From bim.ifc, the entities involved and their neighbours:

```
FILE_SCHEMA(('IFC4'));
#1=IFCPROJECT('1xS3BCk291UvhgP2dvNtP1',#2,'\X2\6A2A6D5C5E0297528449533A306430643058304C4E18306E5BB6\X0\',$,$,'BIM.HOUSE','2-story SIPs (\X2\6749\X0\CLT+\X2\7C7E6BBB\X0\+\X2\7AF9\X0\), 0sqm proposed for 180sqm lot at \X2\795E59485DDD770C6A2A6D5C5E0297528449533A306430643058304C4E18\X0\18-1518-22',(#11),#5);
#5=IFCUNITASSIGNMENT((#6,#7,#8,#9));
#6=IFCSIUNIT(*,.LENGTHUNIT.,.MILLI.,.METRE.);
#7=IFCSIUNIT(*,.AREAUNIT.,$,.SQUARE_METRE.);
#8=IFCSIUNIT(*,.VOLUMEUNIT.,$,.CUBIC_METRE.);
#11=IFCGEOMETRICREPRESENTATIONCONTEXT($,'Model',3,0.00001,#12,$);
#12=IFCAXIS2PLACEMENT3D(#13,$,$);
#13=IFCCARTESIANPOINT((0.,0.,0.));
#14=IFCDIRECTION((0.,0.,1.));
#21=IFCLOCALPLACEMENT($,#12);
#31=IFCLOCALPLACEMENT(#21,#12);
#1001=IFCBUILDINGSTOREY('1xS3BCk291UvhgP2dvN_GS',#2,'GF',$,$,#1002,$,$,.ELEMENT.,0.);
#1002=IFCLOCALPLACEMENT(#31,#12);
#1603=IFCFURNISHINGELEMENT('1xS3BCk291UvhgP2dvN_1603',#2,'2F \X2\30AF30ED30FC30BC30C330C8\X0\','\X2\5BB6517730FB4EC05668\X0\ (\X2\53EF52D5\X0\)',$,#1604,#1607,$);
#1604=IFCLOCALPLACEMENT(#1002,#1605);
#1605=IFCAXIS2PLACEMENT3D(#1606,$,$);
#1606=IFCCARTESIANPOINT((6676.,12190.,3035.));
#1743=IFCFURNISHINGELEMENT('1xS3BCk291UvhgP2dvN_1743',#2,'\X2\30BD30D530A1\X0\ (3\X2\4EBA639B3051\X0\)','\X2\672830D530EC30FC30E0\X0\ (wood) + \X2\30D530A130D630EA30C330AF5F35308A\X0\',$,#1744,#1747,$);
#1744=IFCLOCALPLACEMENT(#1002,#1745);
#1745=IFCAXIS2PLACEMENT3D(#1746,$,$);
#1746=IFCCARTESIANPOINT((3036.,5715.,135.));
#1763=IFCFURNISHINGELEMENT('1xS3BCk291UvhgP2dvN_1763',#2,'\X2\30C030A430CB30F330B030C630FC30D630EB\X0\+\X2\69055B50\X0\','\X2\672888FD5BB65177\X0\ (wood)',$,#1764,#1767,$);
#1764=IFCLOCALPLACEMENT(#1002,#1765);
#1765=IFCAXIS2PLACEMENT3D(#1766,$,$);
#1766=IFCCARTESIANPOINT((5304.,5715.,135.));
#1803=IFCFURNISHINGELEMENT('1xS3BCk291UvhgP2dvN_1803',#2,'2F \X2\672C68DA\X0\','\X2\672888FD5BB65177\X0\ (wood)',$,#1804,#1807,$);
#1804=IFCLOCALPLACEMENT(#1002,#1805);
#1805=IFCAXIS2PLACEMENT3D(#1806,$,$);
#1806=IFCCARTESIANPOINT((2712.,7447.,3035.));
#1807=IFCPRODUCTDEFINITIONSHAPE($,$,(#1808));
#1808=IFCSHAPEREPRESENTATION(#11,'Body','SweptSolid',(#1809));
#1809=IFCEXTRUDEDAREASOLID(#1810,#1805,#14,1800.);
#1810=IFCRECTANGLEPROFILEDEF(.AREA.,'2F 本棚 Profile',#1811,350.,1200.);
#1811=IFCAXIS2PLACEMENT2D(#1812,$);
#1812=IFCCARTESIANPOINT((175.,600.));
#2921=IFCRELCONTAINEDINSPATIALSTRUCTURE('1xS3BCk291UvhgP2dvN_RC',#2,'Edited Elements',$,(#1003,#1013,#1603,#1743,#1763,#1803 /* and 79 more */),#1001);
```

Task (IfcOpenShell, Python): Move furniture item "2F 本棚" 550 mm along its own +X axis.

```python
import ifcopenshell
import ifcopenshell.api.geometry
import ifcopenshell.util.placement
import ifcopenshell.util.unit

model = ifcopenshell.open("bim.ifc")
unit_scale = ifcopenshell.util.unit.calculate_unit_scale(model)

item = model.by_guid("1xS3BCk291UvhgP2dvN_1803")
matrix = ifcopenshell.util.placement.get_local_placement(item.ObjectPlacement)
matrix[:3, 3] += matrix[:3, 0] * 0.55 / unit_scale
ifcopenshell.api.geometry.edit_object_placement(model, product=item, matrix=matrix, is_si=False)

print(ifcopenshell.util.placement.get_local_placement(item.ObjectPlacement).round(3) + 0.0)

model.write("bim-out.ifc")
```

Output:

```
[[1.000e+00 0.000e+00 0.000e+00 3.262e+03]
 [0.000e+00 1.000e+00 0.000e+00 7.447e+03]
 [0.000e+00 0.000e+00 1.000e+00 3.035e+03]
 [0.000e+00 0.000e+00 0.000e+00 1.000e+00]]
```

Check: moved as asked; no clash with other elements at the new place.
